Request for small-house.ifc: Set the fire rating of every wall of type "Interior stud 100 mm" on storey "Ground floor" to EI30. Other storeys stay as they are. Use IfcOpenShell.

First a look at what the model holds.

```python
import ifcopenshell
import ifcopenshell.util.element

model = ifcopenshell.open("small-house.ifc")
print(model.schema)
storey = next(s for s in model.by_type("IfcBuildingStorey") if s.Name == "Ground floor")
walls = [e for e in ifcopenshell.util.element.get_decomposition(storey) if e.is_a("IfcWall")]
seen = {}
for e in walls:
    element_type = ifcopenshell.util.element.get_type(e)
    key = (element_type.Name if element_type != e and element_type else None, ifcopenshell.util.element.get_pset(e, "Pset_WallCommon", "FireRating"))
    seen[key] = seen.get(key, 0) + 1
for (name, value), count in sorted(seen.items(), key=str):
    print(count, "x", name, "|", value)
```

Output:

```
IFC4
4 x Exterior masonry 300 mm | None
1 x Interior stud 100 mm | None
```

```python
import ifcopenshell
import ifcopenshell.api.pset
import ifcopenshell.util.element

model = ifcopenshell.open("small-house.ifc")

storey = next(s for s in model.by_type("IfcBuildingStorey") if s.Name == "Ground floor")
walls = [e for e in ifcopenshell.util.element.get_decomposition(storey) if e.is_a("IfcWall")]

count = 0
for e in walls:
    element_type = ifcopenshell.util.element.get_type(e)
    if element_type in (None, e) or element_type.Name != "Interior stud 100 mm":
        continue
    # add_pset returns the element's existing set when there is one.
    pset = ifcopenshell.api.pset.add_pset(model, product=e, name="Pset_WallCommon")
    ifcopenshell.api.pset.edit_pset(model, pset=pset, properties={"FireRating": "EI30"})
    count += 1

print(count, "walls updated")

model.write("small-house-out.ifc")
```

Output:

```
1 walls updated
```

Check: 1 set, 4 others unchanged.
